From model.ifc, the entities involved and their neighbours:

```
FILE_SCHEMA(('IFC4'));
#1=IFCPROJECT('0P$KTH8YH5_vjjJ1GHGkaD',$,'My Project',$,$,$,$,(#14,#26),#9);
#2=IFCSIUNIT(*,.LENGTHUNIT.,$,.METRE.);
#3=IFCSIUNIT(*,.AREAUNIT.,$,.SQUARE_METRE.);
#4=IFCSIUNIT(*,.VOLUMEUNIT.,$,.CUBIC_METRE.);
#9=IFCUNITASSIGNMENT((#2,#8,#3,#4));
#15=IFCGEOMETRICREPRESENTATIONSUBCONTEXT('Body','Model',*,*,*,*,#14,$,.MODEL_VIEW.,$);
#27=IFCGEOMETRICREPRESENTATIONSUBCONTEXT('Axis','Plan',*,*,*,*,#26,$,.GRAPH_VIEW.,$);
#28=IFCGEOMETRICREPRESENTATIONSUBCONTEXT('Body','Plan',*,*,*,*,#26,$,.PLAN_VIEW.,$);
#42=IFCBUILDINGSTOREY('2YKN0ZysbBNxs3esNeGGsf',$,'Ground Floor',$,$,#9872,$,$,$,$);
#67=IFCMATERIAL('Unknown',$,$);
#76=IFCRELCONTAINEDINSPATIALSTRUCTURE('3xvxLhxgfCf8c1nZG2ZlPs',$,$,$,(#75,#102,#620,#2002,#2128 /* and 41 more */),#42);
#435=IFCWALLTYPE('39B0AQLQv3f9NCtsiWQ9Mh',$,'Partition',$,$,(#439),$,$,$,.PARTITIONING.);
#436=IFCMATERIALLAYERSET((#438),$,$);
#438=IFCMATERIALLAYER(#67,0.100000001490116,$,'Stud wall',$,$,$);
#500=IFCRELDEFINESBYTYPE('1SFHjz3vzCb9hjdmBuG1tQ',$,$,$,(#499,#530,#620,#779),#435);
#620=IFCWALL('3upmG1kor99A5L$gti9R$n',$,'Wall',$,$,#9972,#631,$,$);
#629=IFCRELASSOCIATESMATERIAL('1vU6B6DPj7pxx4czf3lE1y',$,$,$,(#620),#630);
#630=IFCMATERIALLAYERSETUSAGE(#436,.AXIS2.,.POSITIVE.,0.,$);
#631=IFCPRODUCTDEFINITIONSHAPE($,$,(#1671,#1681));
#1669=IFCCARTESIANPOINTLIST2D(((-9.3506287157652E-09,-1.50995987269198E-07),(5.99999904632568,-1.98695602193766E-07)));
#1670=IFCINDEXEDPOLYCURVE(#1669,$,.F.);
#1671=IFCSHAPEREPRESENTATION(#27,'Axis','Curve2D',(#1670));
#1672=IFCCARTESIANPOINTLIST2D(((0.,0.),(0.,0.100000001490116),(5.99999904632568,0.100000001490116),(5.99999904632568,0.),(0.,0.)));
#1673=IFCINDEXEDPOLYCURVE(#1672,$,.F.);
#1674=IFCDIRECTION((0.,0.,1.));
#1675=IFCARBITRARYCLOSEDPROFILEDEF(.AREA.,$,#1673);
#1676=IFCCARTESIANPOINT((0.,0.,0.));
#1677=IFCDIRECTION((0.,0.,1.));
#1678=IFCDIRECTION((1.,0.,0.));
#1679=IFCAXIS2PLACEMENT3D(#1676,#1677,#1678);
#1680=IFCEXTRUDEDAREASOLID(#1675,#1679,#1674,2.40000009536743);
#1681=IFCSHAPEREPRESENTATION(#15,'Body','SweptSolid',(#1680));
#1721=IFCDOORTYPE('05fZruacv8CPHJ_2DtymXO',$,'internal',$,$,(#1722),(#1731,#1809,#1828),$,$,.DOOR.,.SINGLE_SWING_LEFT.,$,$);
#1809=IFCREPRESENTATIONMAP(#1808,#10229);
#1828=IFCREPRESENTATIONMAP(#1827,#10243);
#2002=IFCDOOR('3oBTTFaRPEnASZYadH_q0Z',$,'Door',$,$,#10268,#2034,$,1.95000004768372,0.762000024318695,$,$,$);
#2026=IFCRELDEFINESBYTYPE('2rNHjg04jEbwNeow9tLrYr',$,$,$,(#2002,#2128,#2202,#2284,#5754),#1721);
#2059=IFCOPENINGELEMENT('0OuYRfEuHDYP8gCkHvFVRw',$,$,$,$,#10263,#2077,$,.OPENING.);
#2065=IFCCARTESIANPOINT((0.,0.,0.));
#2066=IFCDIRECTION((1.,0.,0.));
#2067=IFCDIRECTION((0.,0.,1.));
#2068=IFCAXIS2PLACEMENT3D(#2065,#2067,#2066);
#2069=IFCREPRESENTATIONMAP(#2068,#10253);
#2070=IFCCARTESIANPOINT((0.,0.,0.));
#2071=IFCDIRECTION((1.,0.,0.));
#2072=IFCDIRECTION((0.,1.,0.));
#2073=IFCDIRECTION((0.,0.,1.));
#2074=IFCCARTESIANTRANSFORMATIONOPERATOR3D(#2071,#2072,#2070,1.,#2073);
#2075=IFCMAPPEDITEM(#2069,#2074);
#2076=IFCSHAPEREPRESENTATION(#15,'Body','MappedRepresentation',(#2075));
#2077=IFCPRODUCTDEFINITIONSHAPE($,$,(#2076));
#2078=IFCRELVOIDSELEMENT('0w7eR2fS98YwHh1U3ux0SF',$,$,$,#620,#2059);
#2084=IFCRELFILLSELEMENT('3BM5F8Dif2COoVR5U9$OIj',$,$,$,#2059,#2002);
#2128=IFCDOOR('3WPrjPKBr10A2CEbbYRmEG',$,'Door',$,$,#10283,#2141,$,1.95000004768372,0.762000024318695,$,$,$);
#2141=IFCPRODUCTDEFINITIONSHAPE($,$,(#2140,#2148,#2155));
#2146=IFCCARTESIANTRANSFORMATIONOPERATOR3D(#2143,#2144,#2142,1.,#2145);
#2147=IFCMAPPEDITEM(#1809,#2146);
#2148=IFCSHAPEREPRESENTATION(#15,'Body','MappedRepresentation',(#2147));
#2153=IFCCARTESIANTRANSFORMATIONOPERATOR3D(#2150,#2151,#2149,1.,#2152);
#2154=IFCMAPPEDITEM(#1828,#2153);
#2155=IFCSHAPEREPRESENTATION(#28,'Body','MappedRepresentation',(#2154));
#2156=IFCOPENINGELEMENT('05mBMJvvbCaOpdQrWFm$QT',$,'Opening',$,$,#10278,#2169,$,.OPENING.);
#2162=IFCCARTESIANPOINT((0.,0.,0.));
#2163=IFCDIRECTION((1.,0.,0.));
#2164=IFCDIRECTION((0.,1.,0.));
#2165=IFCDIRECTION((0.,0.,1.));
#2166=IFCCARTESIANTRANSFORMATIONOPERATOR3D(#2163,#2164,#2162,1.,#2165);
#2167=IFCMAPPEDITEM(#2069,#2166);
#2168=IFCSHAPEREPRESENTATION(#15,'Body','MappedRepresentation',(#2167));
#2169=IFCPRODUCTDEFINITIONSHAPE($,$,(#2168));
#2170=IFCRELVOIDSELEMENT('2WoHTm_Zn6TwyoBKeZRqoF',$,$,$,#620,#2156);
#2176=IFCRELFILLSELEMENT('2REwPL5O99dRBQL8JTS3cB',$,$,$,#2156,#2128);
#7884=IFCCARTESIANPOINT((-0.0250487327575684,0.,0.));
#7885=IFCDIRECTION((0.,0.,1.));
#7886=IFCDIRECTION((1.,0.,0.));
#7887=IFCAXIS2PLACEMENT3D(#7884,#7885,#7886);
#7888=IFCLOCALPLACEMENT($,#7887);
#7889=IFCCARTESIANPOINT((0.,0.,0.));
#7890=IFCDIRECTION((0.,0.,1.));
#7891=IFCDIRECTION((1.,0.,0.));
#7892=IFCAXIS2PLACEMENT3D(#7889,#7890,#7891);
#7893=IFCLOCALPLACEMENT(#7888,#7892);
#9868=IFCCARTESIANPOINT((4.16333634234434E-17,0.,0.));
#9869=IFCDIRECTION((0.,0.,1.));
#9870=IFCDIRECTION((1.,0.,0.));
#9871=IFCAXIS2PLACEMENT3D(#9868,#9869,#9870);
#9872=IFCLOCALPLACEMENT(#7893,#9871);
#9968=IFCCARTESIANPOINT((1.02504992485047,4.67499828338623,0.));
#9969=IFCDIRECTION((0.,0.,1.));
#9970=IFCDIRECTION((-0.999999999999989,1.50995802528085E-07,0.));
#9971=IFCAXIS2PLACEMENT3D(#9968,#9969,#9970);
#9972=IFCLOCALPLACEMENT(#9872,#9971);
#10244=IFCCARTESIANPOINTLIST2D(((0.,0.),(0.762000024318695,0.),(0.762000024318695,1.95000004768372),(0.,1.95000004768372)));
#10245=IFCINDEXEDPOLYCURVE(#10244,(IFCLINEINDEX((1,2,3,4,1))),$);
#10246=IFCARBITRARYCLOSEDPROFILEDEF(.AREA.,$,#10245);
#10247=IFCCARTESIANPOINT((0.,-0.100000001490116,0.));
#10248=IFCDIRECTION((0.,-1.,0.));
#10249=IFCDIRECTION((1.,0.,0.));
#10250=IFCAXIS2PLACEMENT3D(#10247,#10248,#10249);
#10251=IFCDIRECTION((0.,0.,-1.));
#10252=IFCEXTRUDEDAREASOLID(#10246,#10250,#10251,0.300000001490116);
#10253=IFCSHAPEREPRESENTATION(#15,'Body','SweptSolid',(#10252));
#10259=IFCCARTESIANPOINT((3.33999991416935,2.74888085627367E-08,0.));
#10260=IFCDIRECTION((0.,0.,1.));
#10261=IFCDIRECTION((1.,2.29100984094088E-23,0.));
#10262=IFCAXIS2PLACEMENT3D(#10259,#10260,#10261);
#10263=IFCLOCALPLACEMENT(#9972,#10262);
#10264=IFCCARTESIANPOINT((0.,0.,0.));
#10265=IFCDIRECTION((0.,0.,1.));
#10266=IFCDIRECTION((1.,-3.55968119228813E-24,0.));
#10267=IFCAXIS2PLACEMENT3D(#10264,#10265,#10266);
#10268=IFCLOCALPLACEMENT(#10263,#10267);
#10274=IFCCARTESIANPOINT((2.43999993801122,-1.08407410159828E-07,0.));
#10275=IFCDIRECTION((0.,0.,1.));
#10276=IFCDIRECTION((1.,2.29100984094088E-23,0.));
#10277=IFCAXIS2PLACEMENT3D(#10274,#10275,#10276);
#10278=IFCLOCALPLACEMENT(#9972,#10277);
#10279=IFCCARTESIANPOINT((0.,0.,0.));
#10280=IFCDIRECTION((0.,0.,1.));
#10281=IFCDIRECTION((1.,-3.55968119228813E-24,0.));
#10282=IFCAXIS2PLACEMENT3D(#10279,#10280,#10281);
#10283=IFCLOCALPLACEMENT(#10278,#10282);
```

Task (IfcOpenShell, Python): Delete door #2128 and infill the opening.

```python
import ifcopenshell
import ifcopenshell.api.feature
import ifcopenshell.api.root
import ifcopenshell.geom
import ifcopenshell.util.shape

model = ifcopenshell.open("model.ifc")
settings = ifcopenshell.geom.settings()


def volume(element):
    """Net volume in cubic metres, openings subtracted."""
    shape = ifcopenshell.geom.create_shape(settings, element)
    return ifcopenshell.util.shape.get_volume(shape.geometry)


door = model.by_guid("3WPrjPKBr10A2CEbbYRmEG")
opening = door.FillsVoids[0].RelatingOpeningElement
wall = opening.VoidsElements[0].RelatingBuildingElement
before = volume(wall)

ifcopenshell.api.root.remove_product(model, product=door)
ifcopenshell.api.feature.remove_feature(model, feature=opening)

after = volume(wall)

print(f"wall volume {before:.3f} -> {after:.3f} m3")

model.write("model_v2.ifc")
```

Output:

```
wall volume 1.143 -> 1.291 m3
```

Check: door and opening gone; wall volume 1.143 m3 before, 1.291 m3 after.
